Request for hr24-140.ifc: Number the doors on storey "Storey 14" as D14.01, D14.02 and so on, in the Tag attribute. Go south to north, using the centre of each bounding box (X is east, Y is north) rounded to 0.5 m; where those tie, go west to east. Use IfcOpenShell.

First a look at what the model holds.

```python
import ifcopenshell
import ifcopenshell.util.element
import ifcopenshell.util.placement

model = ifcopenshell.open("hr24-140.ifc")
print(model.schema)
storey = next(s for s in model.by_type("IfcBuildingStorey") if s.Name == "Storey 14")
doors = [e for e in ifcopenshell.util.element.get_decomposition(storey) if e.is_a("IfcDoor")]
for e in sorted(doors, key=lambda e: e.id()):
    origin = ifcopenshell.util.placement.get_local_placement(e.ObjectPlacement)[:3, 3]
    print(e.id(), e.Tag, e.Name, origin.round(2) + 0.0, sep=" | ")
```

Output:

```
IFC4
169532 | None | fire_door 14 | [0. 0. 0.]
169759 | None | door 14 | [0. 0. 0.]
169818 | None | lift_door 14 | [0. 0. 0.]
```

```python
import ifcopenshell
import ifcopenshell.geom
import ifcopenshell.util.element
import ifcopenshell.util.shape

model = ifcopenshell.open("hr24-140.ifc")
settings = ifcopenshell.geom.settings()
settings.set("use-world-coords", True)


def centre(element):
    shape = ifcopenshell.geom.create_shape(settings, element)
    return ifcopenshell.util.shape.get_bbox_centroid(shape.geometry)


storey = next(s for s in model.by_type("IfcBuildingStorey") if s.Name == "Storey 14")
doors = [e for e in ifcopenshell.util.element.get_decomposition(storey) if e.is_a("IfcDoor")]

# Insertion points can sit at a corner or the storey origin, so sort by the geometry (in metres).
centres = {e: centre(e) for e in doors}
doors.sort(key=lambda e: (round(centres[e][1] / 0.5), centres[e][0]))

for i, e in enumerate(doors, start=1):
    number = f"D14.{i:02d}"
    e.Tag = number
    print(e.id(), number)

model.write("hr24-140_rev.ifc")
```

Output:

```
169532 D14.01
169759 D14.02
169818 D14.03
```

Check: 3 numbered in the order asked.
